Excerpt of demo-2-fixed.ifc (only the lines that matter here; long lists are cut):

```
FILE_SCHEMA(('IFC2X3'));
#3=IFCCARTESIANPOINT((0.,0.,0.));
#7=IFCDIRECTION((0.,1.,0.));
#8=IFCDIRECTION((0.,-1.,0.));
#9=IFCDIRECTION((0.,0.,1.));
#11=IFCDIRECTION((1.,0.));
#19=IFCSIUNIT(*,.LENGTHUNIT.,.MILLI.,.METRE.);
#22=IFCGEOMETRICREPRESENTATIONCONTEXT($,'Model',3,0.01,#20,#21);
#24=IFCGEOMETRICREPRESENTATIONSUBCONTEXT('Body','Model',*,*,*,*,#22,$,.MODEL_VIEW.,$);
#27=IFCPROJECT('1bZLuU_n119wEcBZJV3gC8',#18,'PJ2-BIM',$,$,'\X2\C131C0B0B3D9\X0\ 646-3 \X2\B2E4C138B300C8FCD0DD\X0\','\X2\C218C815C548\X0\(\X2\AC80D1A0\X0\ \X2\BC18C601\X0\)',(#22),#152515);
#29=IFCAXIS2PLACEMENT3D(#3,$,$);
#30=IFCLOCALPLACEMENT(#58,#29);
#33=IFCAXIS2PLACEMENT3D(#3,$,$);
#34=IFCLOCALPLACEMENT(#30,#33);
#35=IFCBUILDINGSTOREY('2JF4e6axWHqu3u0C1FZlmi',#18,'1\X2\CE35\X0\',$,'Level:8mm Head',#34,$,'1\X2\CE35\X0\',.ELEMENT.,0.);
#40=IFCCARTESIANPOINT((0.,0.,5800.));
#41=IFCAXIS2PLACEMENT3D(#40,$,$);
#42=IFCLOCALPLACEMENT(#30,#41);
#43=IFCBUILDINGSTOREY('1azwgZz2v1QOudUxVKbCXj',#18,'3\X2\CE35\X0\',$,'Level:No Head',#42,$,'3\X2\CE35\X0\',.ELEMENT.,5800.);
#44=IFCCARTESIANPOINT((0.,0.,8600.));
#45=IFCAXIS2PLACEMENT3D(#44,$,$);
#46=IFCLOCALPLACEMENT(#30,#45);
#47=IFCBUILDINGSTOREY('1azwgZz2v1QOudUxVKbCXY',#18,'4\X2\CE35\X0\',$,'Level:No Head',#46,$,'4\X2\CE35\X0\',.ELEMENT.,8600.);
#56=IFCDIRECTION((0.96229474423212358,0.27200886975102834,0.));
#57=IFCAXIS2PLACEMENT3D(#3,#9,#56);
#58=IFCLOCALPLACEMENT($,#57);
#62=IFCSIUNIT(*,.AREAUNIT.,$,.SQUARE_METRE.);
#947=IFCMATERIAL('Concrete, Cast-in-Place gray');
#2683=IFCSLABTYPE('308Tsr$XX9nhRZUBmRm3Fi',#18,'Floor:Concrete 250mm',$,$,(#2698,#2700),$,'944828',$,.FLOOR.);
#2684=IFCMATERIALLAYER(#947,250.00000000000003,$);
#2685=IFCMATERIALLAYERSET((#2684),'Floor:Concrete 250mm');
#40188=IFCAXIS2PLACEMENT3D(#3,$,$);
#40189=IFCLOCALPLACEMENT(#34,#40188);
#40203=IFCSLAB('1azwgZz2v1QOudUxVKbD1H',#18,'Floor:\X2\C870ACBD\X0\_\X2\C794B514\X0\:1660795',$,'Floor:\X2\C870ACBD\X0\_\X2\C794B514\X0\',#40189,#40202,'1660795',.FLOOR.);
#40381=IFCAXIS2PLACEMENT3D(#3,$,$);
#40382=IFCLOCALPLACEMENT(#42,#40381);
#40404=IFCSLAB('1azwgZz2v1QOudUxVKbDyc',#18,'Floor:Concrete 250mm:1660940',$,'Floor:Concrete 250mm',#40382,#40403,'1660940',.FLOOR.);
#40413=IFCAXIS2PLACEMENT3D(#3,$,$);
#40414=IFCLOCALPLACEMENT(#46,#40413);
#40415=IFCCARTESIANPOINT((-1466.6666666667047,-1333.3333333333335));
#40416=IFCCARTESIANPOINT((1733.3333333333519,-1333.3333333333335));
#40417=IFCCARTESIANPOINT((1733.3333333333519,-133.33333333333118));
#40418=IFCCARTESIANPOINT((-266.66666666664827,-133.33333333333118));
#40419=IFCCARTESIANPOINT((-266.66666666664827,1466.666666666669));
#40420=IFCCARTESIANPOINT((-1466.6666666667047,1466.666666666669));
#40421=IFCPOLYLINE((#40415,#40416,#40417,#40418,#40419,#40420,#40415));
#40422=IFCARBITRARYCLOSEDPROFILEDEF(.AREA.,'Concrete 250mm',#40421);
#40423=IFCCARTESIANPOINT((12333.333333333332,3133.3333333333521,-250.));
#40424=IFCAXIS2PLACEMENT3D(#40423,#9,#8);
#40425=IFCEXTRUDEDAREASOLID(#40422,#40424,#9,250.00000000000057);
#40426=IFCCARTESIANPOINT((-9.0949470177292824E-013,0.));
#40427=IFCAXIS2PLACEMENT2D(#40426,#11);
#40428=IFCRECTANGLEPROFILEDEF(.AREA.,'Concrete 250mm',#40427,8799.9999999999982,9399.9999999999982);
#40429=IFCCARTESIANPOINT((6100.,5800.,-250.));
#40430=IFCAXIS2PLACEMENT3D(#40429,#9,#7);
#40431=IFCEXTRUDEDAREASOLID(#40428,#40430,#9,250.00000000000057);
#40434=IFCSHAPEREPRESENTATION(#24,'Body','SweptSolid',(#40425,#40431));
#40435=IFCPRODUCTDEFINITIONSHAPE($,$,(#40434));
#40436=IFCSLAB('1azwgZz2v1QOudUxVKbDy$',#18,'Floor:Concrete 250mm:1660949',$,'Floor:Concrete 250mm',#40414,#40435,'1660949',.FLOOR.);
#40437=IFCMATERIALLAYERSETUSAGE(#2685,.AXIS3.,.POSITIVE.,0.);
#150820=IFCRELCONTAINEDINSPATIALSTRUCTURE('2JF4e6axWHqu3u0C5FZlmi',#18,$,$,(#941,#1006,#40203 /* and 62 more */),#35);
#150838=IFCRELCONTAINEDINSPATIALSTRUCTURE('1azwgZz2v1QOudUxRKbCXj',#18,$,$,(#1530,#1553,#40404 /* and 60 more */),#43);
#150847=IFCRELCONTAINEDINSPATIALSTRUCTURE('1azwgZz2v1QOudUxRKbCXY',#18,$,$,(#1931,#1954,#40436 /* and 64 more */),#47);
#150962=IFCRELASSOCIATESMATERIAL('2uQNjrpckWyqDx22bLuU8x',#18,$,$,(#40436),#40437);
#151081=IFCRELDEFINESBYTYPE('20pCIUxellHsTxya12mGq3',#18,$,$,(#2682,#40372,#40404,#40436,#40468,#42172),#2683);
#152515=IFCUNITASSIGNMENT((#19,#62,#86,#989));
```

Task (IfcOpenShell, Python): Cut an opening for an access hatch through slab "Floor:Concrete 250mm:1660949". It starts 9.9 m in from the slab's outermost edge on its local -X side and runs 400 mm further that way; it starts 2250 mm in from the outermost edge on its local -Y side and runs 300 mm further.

```python
import numpy as np
import ifcopenshell
import ifcopenshell.api.feature
import ifcopenshell.api.geometry
import ifcopenshell.api.root
import ifcopenshell.geom
import ifcopenshell.util.placement
import ifcopenshell.util.representation
import ifcopenshell.util.shape
import ifcopenshell.util.unit

model = ifcopenshell.open("demo-2-fixed.ifc")
unit_scale = ifcopenshell.util.unit.calculate_unit_scale(model)
settings = ifcopenshell.geom.settings()


def volume(element):
    """Net volume in cubic metres, openings subtracted."""
    shape = ifcopenshell.geom.create_shape(settings, element)
    return ifcopenshell.util.shape.get_volume(shape.geometry)


slab = model.by_guid("1azwgZz2v1QOudUxVKbDy$")
before = volume(slab)

# Extent in the slab's own axes, in metres. The edges named are its -X and -Y sides.
slab_shape = ifcopenshell.geom.create_shape(settings, slab)
vertices = ifcopenshell.util.shape.get_vertices(slab_shape.geometry)
x_min, y_min, bottom = vertices.min(axis=0)
top = vertices[:, 2].max()

opening = ifcopenshell.api.root.create_entity(model, ifc_class="IfcOpeningElement", name="Access hatch opening")
context = ifcopenshell.util.representation.get_context(model, "Model", "Body", "MODEL_VIEW")
width, depth = 0.4, 0.3
outline = [(0.0, 0.0), (width, 0.0), (width, depth), (0.0, depth), (0.0, 0.0)]
# Overshoot both faces by 50 mm so the cut is clean.
shape = ifcopenshell.api.geometry.add_slab_representation(
    model, context=context, depth=top - bottom + 0.1, polyline=outline
)
ifcopenshell.api.geometry.assign_representation(model, product=opening, representation=shape)

matrix = ifcopenshell.util.placement.get_local_placement(slab.ObjectPlacement)
matrix[:, 3] = matrix @ np.append(np.array([x_min + 9.9, y_min + 2.25, bottom - 0.05]) / unit_scale, 1.0)
ifcopenshell.api.geometry.edit_object_placement(model, product=opening, matrix=matrix, is_si=False)
ifcopenshell.api.feature.add_feature(model, feature=opening, element=slab)

after = volume(slab)

print(f"slab volume {before:.3f} -> {after:.3f} m3")

model.write("demo-2-fixed_edited.ifc")
```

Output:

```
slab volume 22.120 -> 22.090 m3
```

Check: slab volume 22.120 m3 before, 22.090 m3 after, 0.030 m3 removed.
